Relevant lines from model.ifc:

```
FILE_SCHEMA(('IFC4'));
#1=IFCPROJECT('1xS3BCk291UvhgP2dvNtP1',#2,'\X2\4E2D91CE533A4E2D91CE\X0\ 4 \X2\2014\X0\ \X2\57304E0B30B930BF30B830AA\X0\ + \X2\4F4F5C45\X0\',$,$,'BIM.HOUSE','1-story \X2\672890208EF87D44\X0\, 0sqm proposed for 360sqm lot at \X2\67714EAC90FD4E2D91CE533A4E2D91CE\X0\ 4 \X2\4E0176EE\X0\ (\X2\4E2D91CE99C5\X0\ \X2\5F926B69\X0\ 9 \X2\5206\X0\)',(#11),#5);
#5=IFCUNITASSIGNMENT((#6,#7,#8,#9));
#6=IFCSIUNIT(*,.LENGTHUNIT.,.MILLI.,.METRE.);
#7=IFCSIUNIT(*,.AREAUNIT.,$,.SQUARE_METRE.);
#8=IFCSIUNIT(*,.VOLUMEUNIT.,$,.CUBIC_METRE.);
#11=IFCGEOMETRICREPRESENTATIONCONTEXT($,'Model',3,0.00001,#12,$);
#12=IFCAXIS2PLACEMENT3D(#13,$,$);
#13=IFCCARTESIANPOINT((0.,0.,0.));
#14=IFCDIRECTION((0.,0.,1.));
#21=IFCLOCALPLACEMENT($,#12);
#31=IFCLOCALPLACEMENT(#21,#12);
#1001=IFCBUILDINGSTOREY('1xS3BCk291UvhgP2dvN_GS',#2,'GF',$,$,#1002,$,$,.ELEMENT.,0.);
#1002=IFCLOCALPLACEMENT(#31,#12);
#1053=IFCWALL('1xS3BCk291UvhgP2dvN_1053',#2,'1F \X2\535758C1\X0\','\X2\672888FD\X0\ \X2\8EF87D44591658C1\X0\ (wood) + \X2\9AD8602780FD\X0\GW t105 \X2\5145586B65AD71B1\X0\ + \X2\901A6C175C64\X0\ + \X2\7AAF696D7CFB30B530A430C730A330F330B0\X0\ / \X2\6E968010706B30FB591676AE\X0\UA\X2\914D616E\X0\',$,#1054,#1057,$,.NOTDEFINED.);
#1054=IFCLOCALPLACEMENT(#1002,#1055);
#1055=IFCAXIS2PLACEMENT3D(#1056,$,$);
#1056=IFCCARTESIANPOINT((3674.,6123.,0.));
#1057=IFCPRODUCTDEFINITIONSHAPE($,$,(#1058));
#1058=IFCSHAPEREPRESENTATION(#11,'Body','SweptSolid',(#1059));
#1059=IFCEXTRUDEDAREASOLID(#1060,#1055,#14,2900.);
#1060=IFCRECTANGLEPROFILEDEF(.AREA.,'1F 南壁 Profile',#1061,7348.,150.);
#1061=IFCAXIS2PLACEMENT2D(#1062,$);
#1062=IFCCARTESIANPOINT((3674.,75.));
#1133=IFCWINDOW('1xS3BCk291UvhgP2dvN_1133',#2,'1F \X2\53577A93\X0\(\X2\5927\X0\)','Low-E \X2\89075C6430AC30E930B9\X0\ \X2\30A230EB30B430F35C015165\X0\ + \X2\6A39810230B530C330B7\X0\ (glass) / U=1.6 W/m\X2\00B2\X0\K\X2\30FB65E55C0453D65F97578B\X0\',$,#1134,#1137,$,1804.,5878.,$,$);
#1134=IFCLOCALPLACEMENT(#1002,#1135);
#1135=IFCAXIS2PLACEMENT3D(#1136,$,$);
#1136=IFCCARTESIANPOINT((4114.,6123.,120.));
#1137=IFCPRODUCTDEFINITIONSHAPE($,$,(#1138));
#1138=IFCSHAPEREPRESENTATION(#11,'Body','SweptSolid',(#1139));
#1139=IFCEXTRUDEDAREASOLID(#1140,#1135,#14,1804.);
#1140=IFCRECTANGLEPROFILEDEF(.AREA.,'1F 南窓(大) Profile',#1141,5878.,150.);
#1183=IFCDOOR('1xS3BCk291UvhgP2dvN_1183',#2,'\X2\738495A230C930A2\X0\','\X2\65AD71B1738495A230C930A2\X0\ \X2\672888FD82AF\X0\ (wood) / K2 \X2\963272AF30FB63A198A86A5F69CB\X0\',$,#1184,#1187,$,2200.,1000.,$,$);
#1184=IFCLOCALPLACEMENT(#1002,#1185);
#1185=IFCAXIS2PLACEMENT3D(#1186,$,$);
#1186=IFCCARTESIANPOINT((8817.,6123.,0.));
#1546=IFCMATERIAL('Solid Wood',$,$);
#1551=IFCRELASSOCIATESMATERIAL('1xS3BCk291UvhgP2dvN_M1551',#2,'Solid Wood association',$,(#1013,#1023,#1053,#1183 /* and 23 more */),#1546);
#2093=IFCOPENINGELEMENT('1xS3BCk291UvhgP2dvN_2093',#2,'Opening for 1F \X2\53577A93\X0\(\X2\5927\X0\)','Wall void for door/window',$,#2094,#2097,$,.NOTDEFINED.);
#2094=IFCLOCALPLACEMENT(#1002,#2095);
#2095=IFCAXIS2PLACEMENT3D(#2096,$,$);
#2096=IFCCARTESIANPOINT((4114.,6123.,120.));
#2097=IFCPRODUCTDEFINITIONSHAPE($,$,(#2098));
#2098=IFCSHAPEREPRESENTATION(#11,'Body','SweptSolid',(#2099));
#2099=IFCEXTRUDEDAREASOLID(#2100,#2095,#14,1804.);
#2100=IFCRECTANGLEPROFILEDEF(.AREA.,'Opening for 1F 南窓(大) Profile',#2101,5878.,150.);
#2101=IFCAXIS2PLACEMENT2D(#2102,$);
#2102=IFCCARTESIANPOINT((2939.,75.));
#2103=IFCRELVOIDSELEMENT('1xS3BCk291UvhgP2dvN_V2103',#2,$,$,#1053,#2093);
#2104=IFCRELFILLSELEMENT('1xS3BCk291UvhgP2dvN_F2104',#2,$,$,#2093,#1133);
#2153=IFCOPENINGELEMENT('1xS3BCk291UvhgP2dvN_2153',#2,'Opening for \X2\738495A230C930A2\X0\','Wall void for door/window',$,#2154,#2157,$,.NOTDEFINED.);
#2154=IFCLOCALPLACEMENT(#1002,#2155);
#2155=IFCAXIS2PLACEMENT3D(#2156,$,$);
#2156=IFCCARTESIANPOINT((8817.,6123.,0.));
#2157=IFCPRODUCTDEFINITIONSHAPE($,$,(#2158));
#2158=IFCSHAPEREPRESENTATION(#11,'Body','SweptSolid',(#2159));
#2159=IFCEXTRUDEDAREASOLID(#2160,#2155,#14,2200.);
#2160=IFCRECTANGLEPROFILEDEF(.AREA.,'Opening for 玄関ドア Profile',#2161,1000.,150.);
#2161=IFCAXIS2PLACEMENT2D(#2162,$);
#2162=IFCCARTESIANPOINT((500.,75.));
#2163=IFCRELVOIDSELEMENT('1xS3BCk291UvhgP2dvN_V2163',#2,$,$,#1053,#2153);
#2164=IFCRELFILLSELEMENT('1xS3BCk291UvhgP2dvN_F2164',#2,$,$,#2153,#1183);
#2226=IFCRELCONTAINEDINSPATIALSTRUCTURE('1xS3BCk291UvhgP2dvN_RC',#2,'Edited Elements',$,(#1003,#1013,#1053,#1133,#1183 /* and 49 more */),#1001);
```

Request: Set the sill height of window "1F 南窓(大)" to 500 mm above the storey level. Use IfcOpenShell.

```python
import numpy as np
import ifcopenshell
import ifcopenshell.api.geometry
import ifcopenshell.geom
import ifcopenshell.util.element
import ifcopenshell.util.placement
import ifcopenshell.util.shape
import ifcopenshell.util.unit

model = ifcopenshell.open("model.ifc")
unit_scale = ifcopenshell.util.unit.calculate_unit_scale(model)

window = model.by_id(1133)
opening = window.FillsVoids[0].RelatingOpeningElement
storey = ifcopenshell.util.element.get_container(window, ifc_class="IfcBuildingStorey")
level = ifcopenshell.util.placement.get_local_placement(storey.ObjectPlacement)[2, 3]

# The opening's origin need not be at the sill, so measure its lowest point.
shape = ifcopenshell.geom.create_shape(ifcopenshell.geom.settings(), opening)
bottom = ifcopenshell.util.shape.get_shape_bottom_elevation(shape, shape.geometry) / unit_scale
dz = level + 500.0 - bottom

shift = np.array([0.0, 0.0, dz])
# The window is not placed relative to its opening, so move both.
for product in (opening, window):
    matrix = ifcopenshell.util.placement.get_local_placement(product.ObjectPlacement)
    matrix[:3, 3] += shift
    ifcopenshell.api.geometry.edit_object_placement(model, product=product, matrix=matrix, is_si=False)

print(f"moved by {dz * unit_scale:+.3f} m")

model.write("model_rev.ifc")
```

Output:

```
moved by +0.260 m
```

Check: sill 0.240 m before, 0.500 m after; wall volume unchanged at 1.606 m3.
